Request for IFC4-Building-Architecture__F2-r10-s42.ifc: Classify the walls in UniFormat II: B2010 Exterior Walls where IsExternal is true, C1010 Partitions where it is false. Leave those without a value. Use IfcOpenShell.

First a look at what the model holds.

```python
import ifcopenshell
import ifcopenshell.util.element

model = ifcopenshell.open("IFC4-Building-Architecture__F2-r10-s42.ifc")
print(model.schema)
print("classifications:", [c.Name for c in model.by_type("IfcClassification")])
values = [ifcopenshell.util.element.get_pset(e, "Pset_WallCommon", "IsExternal") for e in model.by_type("IfcWall")]
for value in (True, False, None):
    print("IsExternal", value, values.count(value))
```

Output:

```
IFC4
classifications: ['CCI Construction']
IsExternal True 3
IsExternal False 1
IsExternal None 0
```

```python
import ifcopenshell
import ifcopenshell.api.classification
import ifcopenshell.util.element

model = ifcopenshell.open("IFC4-Building-Architecture__F2-r10-s42.ifc")

system = ifcopenshell.api.classification.add_classification(model, classification="UniFormat II")

walls = model.by_type("IfcWall")
external = {e: ifcopenshell.util.element.get_pset(e, "Pset_WallCommon", "IsExternal") for e in walls}
for flag, code, name in ((True, "B2010", "Exterior Walls"), (False, "C1010", "Partitions")):
    products = [e for e in walls if external[e] is flag]
    ifcopenshell.api.classification.add_reference(
        model, products=products, classification=system, identification=code, name=name
    )
    print(code, len(products))

model.write("IFC4-Building-Architecture__F2-r10-s42_edited.ifc")
```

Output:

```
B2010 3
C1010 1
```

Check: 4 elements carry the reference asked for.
